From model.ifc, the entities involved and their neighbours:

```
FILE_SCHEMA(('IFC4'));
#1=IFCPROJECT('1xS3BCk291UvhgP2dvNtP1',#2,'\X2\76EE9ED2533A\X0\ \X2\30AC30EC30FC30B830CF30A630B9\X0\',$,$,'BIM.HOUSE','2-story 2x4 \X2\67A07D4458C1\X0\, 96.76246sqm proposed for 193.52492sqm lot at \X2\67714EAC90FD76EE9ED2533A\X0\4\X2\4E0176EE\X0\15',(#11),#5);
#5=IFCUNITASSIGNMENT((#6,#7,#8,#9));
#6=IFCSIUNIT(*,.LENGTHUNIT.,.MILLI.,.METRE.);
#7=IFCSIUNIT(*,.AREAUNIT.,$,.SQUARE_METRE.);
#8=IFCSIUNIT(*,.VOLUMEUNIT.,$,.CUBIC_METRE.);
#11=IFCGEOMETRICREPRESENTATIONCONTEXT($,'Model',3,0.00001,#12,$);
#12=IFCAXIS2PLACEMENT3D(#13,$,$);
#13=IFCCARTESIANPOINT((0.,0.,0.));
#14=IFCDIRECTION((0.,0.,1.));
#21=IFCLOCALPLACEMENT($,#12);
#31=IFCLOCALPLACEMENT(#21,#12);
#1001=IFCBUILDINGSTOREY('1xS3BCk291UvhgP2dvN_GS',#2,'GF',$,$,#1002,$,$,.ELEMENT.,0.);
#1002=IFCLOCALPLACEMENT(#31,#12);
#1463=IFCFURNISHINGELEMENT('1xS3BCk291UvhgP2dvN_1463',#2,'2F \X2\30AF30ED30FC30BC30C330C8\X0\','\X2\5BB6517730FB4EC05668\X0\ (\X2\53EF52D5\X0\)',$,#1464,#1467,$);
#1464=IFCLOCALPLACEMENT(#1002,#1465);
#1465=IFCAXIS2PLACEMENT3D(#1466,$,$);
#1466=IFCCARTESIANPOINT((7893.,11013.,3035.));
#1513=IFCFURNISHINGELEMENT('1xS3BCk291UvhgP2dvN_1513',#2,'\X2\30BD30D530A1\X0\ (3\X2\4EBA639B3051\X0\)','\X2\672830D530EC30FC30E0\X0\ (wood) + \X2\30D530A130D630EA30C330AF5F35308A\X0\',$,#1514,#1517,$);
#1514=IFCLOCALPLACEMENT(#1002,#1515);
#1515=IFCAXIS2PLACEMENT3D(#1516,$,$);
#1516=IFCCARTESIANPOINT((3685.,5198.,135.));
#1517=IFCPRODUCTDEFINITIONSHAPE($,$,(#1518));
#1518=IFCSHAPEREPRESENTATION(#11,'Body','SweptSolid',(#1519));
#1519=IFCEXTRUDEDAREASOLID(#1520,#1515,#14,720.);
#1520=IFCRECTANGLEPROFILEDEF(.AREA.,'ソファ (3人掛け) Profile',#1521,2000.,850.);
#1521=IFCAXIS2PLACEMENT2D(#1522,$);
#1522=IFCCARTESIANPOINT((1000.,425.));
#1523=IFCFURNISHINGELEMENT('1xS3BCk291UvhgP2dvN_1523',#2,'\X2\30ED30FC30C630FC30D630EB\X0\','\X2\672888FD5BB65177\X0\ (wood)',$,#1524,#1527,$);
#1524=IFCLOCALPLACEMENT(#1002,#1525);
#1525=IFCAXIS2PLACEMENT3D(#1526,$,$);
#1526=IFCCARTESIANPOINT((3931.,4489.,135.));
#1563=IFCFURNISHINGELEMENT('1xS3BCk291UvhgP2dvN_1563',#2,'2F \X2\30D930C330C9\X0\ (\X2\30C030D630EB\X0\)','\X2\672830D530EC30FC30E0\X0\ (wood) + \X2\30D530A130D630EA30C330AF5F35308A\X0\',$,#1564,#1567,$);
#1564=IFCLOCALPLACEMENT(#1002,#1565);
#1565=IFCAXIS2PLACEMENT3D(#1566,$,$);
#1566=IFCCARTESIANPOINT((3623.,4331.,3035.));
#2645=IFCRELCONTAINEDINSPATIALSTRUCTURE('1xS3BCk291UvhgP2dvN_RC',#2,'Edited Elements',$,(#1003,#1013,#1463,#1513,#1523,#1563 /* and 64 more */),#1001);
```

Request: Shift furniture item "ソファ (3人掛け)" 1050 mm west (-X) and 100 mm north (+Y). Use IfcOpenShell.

```python
import ifcopenshell
import ifcopenshell.api.geometry
import ifcopenshell.util.placement
import ifcopenshell.util.unit

model = ifcopenshell.open("model.ifc")
unit_scale = ifcopenshell.util.unit.calculate_unit_scale(model)

item = model.by_guid("1xS3BCk291UvhgP2dvN_1513")
matrix = ifcopenshell.util.placement.get_local_placement(item.ObjectPlacement)
matrix[0, 3] -= 1.05 / unit_scale
matrix[1, 3] += 0.1 / unit_scale
ifcopenshell.api.geometry.edit_object_placement(model, product=item, matrix=matrix, is_si=False)

print(ifcopenshell.util.placement.get_local_placement(item.ObjectPlacement).round(3) + 0.0)

model.write("model_v2.ifc")
```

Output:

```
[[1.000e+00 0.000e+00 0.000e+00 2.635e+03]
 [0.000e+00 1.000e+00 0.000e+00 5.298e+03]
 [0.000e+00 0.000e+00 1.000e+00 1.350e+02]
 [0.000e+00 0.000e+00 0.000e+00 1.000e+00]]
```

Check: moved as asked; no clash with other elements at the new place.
